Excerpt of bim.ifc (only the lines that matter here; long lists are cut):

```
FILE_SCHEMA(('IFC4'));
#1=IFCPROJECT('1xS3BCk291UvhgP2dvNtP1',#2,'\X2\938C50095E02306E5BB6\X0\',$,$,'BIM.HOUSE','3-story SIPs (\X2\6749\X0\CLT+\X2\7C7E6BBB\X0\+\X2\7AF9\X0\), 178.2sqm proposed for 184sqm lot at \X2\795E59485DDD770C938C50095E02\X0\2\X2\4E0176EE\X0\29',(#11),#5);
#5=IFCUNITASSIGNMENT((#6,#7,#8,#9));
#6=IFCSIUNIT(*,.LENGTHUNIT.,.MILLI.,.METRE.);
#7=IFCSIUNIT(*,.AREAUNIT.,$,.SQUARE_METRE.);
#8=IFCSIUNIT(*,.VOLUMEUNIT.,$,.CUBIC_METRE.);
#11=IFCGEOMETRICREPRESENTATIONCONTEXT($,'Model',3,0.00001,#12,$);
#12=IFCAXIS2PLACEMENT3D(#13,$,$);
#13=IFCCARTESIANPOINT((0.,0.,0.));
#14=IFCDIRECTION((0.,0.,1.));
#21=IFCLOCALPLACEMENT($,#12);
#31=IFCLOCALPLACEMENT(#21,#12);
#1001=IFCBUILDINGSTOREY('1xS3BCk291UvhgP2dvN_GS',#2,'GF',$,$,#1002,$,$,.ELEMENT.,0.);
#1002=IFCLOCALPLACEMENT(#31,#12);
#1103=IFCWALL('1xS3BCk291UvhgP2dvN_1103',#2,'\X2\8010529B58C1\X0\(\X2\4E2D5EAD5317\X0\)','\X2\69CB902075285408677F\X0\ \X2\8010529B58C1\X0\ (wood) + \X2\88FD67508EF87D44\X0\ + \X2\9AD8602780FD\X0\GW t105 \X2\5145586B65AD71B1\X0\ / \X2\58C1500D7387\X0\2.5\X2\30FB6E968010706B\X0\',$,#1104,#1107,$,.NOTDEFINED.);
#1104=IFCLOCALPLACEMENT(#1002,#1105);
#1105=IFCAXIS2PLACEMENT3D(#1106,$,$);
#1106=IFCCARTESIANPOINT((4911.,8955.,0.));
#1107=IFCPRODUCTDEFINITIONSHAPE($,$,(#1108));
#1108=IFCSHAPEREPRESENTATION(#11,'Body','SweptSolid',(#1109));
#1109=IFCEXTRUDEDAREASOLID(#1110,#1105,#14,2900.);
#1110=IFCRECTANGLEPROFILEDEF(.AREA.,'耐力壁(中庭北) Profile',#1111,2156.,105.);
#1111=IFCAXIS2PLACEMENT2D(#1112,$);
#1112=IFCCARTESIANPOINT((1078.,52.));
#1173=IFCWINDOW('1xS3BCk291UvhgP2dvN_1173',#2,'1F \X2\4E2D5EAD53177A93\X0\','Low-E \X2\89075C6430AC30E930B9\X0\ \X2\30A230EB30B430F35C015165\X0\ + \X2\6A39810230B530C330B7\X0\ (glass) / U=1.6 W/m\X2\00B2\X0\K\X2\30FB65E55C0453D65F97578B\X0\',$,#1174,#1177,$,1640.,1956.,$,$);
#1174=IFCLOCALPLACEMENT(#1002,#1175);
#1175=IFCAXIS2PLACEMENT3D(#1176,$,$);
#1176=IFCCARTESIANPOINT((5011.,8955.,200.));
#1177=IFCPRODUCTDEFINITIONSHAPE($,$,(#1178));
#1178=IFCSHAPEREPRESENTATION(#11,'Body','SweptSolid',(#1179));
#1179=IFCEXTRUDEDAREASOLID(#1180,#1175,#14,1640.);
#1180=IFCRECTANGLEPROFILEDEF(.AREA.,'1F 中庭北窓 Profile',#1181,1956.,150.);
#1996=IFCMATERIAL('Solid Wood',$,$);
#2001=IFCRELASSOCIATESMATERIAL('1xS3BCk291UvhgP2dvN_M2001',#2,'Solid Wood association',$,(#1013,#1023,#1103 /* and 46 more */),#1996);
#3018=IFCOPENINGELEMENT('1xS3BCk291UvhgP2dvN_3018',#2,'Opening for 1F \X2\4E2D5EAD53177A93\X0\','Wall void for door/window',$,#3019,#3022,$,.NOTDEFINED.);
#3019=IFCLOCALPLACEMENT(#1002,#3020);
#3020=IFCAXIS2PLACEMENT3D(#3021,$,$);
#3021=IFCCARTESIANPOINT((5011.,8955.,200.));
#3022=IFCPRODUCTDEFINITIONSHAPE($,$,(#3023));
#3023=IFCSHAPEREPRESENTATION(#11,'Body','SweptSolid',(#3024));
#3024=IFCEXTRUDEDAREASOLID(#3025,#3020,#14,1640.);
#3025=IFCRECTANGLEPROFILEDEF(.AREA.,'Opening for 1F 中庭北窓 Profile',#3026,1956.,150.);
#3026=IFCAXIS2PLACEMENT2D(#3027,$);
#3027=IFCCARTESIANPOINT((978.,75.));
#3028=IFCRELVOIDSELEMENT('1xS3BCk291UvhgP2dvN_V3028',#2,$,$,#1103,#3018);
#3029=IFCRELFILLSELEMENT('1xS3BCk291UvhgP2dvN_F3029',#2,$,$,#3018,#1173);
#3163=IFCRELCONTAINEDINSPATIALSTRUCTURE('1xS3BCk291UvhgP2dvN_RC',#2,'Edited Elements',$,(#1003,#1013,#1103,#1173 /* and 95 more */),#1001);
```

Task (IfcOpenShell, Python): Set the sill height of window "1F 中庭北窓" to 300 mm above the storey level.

```python
import numpy as np
import ifcopenshell
import ifcopenshell.api.geometry
import ifcopenshell.geom
import ifcopenshell.util.element
import ifcopenshell.util.placement
import ifcopenshell.util.shape
import ifcopenshell.util.unit

model = ifcopenshell.open("bim.ifc")
unit_scale = ifcopenshell.util.unit.calculate_unit_scale(model)

window = model.by_guid("1xS3BCk291UvhgP2dvN_1173")
opening = window.FillsVoids[0].RelatingOpeningElement
storey = ifcopenshell.util.element.get_container(window, ifc_class="IfcBuildingStorey")
level = ifcopenshell.util.placement.get_local_placement(storey.ObjectPlacement)[2, 3]

# The opening's origin need not be at the sill, so measure its lowest point.
shape = ifcopenshell.geom.create_shape(ifcopenshell.geom.settings(), opening)
bottom = ifcopenshell.util.shape.get_shape_bottom_elevation(shape, shape.geometry) / unit_scale
dz = level + 300.0 - bottom

shift = np.array([0.0, 0.0, dz])
# The window is not placed relative to its opening, so move both.
for product in (opening, window):
    matrix = ifcopenshell.util.placement.get_local_placement(product.ObjectPlacement)
    matrix[:3, 3] += shift
    ifcopenshell.api.geometry.edit_object_placement(model, product=product, matrix=matrix, is_si=False)

print(f"moved by {dz * unit_scale:+.3f} m")

model.write("bim-out.ifc")
```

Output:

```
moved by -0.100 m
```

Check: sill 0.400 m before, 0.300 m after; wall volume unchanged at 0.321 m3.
